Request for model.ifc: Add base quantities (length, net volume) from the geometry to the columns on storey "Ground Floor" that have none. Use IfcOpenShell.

First a look at what the model holds.

```python
import ifcopenshell
import ifcopenshell.util.element
import ifcopenshell.util.unit

model = ifcopenshell.open("model.ifc")
print(model.schema)
for unit_type in ("LENGTHUNIT", "AREAUNIT", "VOLUMEUNIT"):
    print(unit_type, ifcopenshell.util.unit.calculate_unit_scale(model, unit_type))
storey = next(s for s in model.by_type("IfcBuildingStorey") if s.Name == "Ground Floor")
columns = [e for e in ifcopenshell.util.element.get_decomposition(storey) if e.is_a("IfcColumn")]
for e in sorted(columns, key=lambda e: e.id()):
    print(e.id(), e.is_a(), e.Name, list(ifcopenshell.util.element.get_psets(e, qtos_only=True)), sep=" | ")
```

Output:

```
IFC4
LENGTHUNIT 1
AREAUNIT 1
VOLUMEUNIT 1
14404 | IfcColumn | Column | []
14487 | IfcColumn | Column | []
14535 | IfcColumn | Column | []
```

```python
import ifcopenshell
import ifcopenshell.api.pset
import ifcopenshell.geom
import ifcopenshell.util.element
import ifcopenshell.util.shape
import ifcopenshell.util.unit

model = ifcopenshell.open("model.ifc")
unit_scale = ifcopenshell.util.unit.calculate_unit_scale(model)
volume_scale = ifcopenshell.util.unit.calculate_unit_scale(model, "VOLUMEUNIT")
settings = ifcopenshell.geom.settings()

storey = next(s for s in model.by_type("IfcBuildingStorey") if s.Name == "Ground Floor")
columns = [e for e in ifcopenshell.util.element.get_decomposition(storey) if e.is_a("IfcColumn")]

for e in sorted(columns, key=lambda e: e.id()):
    if ifcopenshell.util.element.get_psets(e, qtos_only=True, should_inherit=False):
        continue
    # Geometry comes back in metres, in the element's own axes.
    shape = ifcopenshell.geom.create_shape(settings, e)
    values = {
        "Length": ifcopenshell.util.shape.get_z(shape.geometry) / unit_scale,
        "NetVolume": ifcopenshell.util.shape.get_volume(shape.geometry) / volume_scale,
    }
    qto = ifcopenshell.api.pset.add_qto(model, product=e, name="Qto_ColumnBaseQuantities")
    ifcopenshell.api.pset.edit_qto(model, qto=qto, properties=values)
    print(e.id(), {k: round(v, 3) for k, v in values.items()})

model.write("model_edited.ifc")
```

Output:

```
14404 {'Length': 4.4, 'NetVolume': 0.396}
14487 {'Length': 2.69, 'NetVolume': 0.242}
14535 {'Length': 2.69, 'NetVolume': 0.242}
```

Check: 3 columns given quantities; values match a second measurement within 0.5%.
